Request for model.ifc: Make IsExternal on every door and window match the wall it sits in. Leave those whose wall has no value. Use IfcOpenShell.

First a look at what the model holds.

```python
import ifcopenshell
import ifcopenshell.util.element

model = ifcopenshell.open("model.ifc")
print(model.schema)
seen = {}
for e in model.by_type("IfcDoor") + model.by_type("IfcWindow"):
    if not e.FillsVoids:
        continue
    host = e.FillsVoids[0].RelatingOpeningElement.VoidsElements[0].RelatingBuildingElement
    own = ifcopenshell.util.element.get_pset(e, f"Pset_{e.is_a()[3:].removesuffix('StandardCase')}Common", "IsExternal")
    wall = ifcopenshell.util.element.get_pset(host, "Pset_WallCommon", "IsExternal")
    seen[e.is_a(), own, wall] = seen.get((e.is_a(), own, wall), 0) + 1
for (cls, own, wall), count in sorted(seen.items(), key=str):
    print(count, cls, "IsExternal:", own, "| host wall:", wall)
```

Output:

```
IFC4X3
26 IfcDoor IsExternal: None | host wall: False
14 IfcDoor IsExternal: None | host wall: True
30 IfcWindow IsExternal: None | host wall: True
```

```python
import ifcopenshell
import ifcopenshell.api.pset
import ifcopenshell.util.element

model = ifcopenshell.open("model.ifc")

count = 0
for ifc_class, pset_name in (("IfcDoor", "Pset_DoorCommon"), ("IfcWindow", "Pset_WindowCommon")):
    for e in model.by_type(ifc_class):
        if not e.FillsVoids:
            continue
        host = e.FillsVoids[0].RelatingOpeningElement.VoidsElements[0].RelatingBuildingElement
        external = ifcopenshell.util.element.get_pset(host, "Pset_WallCommon", "IsExternal")
        if external is None or ifcopenshell.util.element.get_pset(e, pset_name, "IsExternal") == external:
            continue
        pset = ifcopenshell.api.pset.add_pset(model, product=e, name=pset_name)
        ifcopenshell.api.pset.edit_pset(model, pset=pset, properties={"IsExternal": external})
        count += 1

print(count, "updated")

model.write("model_edited.ifc")
```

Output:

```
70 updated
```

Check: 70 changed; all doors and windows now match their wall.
